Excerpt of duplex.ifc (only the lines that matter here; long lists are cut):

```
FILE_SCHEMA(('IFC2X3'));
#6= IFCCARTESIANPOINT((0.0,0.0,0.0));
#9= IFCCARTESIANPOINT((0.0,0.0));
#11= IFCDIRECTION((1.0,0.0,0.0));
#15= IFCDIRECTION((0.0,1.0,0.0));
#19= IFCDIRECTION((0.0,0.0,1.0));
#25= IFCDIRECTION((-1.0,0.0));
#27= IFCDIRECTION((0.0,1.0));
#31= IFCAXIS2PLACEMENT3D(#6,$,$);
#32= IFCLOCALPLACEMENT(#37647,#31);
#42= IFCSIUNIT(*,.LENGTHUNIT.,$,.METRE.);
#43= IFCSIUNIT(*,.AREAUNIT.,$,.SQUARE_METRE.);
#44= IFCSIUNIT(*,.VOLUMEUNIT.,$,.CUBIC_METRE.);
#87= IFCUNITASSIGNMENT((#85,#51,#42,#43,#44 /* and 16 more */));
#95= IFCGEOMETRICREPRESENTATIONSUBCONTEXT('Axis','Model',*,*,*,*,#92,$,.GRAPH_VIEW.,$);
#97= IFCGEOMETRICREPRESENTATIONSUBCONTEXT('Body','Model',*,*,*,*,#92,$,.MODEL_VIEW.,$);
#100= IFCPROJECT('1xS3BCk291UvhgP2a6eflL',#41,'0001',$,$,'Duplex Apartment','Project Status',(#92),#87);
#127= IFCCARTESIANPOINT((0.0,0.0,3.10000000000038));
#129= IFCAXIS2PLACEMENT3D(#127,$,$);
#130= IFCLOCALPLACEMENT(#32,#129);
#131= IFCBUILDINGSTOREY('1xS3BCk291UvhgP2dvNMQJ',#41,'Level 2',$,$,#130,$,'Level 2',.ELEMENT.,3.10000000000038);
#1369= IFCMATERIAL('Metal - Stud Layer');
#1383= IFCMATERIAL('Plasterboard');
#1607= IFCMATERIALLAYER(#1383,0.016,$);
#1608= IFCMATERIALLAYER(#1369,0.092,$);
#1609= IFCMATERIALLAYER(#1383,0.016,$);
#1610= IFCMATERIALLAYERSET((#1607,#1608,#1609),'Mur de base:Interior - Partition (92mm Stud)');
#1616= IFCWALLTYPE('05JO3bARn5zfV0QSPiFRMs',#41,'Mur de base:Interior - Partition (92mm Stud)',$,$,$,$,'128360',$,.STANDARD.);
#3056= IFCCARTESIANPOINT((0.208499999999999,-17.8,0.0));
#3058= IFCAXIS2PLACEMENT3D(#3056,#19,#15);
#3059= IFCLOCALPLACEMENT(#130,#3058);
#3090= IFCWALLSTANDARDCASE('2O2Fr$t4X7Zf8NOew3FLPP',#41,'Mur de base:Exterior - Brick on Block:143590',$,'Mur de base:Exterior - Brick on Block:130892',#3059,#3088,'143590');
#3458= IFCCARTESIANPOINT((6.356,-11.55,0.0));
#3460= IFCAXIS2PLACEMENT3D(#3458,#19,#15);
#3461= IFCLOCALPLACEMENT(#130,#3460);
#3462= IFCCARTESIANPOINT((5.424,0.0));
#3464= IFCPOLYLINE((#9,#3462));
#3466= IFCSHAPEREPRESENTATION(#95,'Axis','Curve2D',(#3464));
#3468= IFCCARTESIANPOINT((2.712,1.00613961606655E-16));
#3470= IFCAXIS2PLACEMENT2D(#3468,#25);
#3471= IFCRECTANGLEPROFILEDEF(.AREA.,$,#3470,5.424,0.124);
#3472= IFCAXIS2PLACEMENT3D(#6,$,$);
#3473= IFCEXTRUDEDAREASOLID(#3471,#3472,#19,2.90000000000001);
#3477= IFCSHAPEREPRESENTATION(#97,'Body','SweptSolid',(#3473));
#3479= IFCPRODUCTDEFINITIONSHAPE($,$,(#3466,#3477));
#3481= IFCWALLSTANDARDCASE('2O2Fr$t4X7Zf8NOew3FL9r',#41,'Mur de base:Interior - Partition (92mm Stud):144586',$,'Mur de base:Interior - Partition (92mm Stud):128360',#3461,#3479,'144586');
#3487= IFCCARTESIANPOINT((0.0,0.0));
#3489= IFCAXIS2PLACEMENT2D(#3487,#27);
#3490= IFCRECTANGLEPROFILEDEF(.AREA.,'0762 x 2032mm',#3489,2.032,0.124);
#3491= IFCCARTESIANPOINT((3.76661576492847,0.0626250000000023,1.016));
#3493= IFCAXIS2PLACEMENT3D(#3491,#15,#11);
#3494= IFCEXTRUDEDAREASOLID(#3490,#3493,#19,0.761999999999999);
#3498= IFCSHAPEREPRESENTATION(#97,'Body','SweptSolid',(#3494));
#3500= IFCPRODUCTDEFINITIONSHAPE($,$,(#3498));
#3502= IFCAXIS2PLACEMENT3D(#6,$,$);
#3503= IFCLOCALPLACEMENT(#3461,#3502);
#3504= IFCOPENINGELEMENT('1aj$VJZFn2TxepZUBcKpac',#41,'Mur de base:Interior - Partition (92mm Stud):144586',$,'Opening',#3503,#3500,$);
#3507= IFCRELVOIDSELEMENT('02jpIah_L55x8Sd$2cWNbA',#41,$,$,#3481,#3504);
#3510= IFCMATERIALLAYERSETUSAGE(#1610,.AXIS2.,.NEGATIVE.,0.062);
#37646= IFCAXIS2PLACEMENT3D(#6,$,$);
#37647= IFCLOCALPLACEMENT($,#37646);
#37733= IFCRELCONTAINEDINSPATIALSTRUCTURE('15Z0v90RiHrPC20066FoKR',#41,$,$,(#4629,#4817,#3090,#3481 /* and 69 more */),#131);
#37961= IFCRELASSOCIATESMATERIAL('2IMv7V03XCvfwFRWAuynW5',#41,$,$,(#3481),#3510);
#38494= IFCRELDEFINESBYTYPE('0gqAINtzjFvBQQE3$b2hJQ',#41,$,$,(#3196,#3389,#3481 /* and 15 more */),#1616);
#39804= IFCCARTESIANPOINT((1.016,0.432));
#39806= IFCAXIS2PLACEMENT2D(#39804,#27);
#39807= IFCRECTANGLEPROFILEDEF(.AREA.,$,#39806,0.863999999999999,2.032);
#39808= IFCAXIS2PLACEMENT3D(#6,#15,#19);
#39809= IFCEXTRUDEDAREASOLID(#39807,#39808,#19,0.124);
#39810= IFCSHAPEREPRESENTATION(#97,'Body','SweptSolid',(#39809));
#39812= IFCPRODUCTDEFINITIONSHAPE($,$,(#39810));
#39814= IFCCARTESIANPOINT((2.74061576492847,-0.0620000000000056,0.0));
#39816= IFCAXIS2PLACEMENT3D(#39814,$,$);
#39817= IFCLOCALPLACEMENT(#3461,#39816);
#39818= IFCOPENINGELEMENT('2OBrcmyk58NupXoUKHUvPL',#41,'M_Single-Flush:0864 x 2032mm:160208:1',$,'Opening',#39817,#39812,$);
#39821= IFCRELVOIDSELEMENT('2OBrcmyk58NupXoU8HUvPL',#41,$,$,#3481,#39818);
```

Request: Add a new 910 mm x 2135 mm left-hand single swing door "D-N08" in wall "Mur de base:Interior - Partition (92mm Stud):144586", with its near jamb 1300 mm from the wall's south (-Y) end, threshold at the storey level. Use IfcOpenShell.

```python
import numpy as np
import ifcopenshell
import ifcopenshell.api.feature
import ifcopenshell.api.geometry
import ifcopenshell.api.root
import ifcopenshell.api.spatial
import ifcopenshell.api.type
import ifcopenshell.geom
import ifcopenshell.util.element
import ifcopenshell.util.placement
import ifcopenshell.util.representation
import ifcopenshell.util.shape
import ifcopenshell.util.unit

model = ifcopenshell.open("duplex.ifc")
unit_scale = ifcopenshell.util.unit.calculate_unit_scale(model)
settings = ifcopenshell.geom.settings()


def volume(element):
    """Net volume in cubic metres, openings subtracted."""
    shape = ifcopenshell.geom.create_shape(settings, element)
    return ifcopenshell.util.shape.get_volume(shape.geometry)


wall = model.by_id(3481)
storey = ifcopenshell.util.element.get_container(wall, ifc_class="IfcBuildingStorey")
context = ifcopenshell.util.representation.get_context(model, "Model", "Body", "MODEL_VIEW")
before = volume(wall)

width, height, from_end, sill = 0.91, 2.135, 1.3, 0.0  # metres

# The wall runs along its own X axis, and the end named is its -X end.
wall_shape = ifcopenshell.geom.create_shape(settings, wall)
x, y, z = ifcopenshell.util.shape.get_vertices(wall_shape.geometry).T
start = x.min() + from_end
face, thickness = float(y.min()), float(y.max() - y.min())
wall_matrix = ifcopenshell.util.placement.get_local_placement(wall.ObjectPlacement)
level = ifcopenshell.util.placement.get_local_placement(storey.ObjectPlacement)[2, 3]


def in_wall(x, y):
    """Placement at x, y metres in the wall's axes, at sill height."""
    matrix = wall_matrix.copy()
    matrix[:, 3] = wall_matrix @ np.array([x / unit_scale, y / unit_scale, 0.0, 1.0])
    matrix[2, 3] = level + sill / unit_scale
    return matrix


# Opening: a box that overshoots both wall faces by 50 mm.
opening = ifcopenshell.api.root.create_entity(model, ifc_class="IfcOpeningElement")
box = ifcopenshell.api.geometry.add_wall_representation(
    model, context=context, length=width, height=height, thickness=thickness + 0.1
)
ifcopenshell.api.geometry.assign_representation(model, product=opening, representation=box)
ifcopenshell.api.geometry.edit_object_placement(model, product=opening, matrix=in_wall(start, face - 0.05), is_si=False)
ifcopenshell.api.feature.add_feature(model, feature=opening, element=wall)

door = ifcopenshell.api.root.create_entity(model, ifc_class="IfcDoor", name="D-N08")
door.OverallWidth, door.OverallHeight = width / unit_scale, height / unit_scale
body = ifcopenshell.api.geometry.add_door_representation(
    model,
    context=context,
    overall_width=door.OverallWidth,
    overall_height=door.OverallHeight,
    operation_type="SINGLE_SWING_LEFT",
    lining_properties={"LiningDepth": thickness / unit_scale, "ThresholdDepth": thickness / unit_scale},
)
ifcopenshell.api.geometry.assign_representation(model, product=door, representation=body)
ifcopenshell.api.spatial.assign_container(model, products=[door], relating_structure=storey)
fills = ifcopenshell.api.feature.add_filling(model, opening=opening, element=door)
fills.OwnerHistory = door.OwnerHistory  # required in IFC2X3

# IFC2X3 keeps the operation on the door style.
style = ifcopenshell.api.root.create_entity(model, ifc_class="IfcDoorStyle", name="D-N08")
style.OperationType, style.ConstructionType = "SINGLE_SWING_LEFT", "NOTDEFINED"
style.ParameterTakesPrecedence = style.Sizeable = False
ifcopenshell.api.type.assign_type(model, related_objects=[door], relating_type=style)

# The lining spans the wall, so the door starts at the wall face.
ifcopenshell.api.geometry.edit_object_placement(model, product=door, matrix=in_wall(start, face), is_si=False)

after = volume(wall)

print(f"wall volume {before:.3f} -> {after:.3f} m3")

model.write("duplex_updated.ifc")
```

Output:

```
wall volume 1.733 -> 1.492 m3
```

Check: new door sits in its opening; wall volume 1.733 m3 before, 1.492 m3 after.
